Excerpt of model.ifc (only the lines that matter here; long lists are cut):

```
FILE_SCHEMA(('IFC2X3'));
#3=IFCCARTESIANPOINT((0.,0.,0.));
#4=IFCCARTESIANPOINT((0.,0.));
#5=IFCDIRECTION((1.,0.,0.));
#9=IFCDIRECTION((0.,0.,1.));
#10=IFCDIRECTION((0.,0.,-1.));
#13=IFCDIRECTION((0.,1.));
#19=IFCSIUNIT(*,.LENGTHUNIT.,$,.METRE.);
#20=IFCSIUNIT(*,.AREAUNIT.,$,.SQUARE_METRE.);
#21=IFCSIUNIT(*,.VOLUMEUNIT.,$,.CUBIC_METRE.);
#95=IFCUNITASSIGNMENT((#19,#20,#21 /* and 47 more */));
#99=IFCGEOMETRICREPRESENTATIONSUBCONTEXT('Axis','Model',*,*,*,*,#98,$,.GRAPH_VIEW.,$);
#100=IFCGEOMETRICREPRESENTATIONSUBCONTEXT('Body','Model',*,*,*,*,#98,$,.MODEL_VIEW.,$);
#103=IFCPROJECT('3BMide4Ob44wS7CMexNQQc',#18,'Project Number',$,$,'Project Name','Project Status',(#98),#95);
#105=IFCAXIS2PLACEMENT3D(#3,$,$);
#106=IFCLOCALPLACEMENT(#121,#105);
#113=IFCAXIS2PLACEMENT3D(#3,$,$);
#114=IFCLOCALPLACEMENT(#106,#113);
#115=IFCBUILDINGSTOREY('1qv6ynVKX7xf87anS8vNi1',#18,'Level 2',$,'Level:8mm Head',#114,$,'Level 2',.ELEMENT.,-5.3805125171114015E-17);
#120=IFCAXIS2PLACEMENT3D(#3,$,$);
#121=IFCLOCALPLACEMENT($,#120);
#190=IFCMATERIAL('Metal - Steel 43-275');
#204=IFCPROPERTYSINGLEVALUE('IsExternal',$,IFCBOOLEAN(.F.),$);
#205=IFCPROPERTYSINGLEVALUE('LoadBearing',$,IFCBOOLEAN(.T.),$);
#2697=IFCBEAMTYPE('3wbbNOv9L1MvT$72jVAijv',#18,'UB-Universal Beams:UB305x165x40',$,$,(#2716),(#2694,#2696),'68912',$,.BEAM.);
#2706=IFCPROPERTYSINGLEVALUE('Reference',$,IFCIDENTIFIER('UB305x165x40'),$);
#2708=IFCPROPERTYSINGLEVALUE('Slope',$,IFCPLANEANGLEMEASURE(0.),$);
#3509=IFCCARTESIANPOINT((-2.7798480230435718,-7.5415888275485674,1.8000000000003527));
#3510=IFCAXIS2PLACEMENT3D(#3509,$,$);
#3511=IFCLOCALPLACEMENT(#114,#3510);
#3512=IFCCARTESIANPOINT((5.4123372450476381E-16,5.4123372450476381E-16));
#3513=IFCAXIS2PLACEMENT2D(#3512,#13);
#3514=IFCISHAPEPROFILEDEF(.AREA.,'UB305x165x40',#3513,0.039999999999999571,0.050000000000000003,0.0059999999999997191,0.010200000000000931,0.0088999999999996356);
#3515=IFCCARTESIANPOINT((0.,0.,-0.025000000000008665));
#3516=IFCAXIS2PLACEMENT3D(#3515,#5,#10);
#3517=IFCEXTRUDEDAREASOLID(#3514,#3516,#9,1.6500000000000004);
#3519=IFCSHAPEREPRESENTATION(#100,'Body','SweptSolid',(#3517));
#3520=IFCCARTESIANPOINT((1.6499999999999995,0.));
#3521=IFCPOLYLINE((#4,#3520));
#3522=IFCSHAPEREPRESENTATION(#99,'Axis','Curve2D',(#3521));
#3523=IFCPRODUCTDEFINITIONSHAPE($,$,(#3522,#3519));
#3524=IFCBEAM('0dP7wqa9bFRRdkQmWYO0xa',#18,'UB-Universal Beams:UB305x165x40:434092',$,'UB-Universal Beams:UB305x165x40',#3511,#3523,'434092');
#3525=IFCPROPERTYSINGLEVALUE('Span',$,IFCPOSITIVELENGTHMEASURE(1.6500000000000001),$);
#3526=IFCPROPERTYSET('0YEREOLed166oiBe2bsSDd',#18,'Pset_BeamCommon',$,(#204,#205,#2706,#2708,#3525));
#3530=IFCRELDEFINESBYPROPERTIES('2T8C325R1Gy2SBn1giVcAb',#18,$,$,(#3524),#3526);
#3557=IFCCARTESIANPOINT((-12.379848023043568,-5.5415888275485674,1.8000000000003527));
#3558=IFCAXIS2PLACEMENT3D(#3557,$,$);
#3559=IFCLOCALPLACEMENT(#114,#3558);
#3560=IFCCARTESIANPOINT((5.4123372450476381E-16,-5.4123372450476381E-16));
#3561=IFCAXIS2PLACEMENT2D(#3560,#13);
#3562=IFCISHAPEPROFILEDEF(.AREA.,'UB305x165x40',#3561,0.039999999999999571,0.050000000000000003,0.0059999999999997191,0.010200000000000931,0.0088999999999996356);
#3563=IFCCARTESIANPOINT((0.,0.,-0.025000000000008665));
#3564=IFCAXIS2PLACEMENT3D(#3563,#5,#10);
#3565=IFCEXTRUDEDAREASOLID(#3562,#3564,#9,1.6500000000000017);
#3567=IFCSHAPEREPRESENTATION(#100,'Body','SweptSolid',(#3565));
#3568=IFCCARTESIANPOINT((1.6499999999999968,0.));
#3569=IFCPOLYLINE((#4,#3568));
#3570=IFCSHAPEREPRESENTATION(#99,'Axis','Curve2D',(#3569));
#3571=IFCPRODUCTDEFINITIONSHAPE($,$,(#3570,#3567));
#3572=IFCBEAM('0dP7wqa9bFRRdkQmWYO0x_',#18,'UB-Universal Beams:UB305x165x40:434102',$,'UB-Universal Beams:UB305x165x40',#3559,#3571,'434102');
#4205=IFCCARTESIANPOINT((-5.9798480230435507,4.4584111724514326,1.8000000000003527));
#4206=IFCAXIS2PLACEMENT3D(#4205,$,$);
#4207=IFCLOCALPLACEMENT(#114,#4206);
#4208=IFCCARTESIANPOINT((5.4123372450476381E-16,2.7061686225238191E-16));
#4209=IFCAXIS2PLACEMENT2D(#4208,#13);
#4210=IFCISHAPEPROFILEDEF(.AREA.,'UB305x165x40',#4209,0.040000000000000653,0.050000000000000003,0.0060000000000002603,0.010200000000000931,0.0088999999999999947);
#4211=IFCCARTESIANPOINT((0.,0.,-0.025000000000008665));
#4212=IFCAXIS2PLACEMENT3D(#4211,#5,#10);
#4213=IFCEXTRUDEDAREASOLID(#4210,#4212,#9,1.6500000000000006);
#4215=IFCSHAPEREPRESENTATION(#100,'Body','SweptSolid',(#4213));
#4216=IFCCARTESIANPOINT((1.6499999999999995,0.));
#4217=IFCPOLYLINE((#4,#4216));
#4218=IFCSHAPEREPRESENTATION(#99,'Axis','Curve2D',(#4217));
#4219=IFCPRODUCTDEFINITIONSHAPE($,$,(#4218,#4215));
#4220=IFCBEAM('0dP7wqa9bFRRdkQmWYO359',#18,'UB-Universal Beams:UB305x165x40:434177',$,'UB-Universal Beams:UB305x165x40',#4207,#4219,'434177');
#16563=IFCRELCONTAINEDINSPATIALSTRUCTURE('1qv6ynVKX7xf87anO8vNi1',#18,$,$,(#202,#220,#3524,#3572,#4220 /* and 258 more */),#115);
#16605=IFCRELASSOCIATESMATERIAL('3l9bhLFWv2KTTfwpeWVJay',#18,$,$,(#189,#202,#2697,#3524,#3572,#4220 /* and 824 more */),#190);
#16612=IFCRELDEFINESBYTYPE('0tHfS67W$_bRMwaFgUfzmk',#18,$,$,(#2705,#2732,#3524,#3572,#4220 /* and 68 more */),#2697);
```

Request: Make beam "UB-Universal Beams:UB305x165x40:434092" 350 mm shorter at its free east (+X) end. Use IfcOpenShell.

```python
import numpy as np
import ifcopenshell
import ifcopenshell.api.pset
import ifcopenshell.util.element
import ifcopenshell.util.representation

model = ifcopenshell.open("model.ifc")

member = model.by_guid("0dP7wqa9bFRRdkQmWYO0xa")
change = -0.35

# The extrusion runs towards the end named, so only its depth changes.
body = ifcopenshell.util.representation.get_representation(member, "Model", "Body")
solid = body.Items[0]
old_length = solid.Depth
solid.Depth += change

# Move the axis end point with it.
axis = next(r for r in member.Representation.Representations if r.RepresentationIdentifier == "Axis").Items[0]
start, end = (np.array(p.Coordinates) for p in axis.Points)
end = end + (end - start) / np.linalg.norm(end - start) * change
point = model.createIfcCartesianPoint(end.tolist())
axis.Points = [axis.Points[0], point]

# Update the stored length and volume.
pset = model.by_id(ifcopenshell.util.element.get_pset(member, "Pset_BeamCommon", should_inherit=False)["id"])
ifcopenshell.api.pset.edit_pset(model, pset=pset, properties={
    "Span": model.create_entity("IfcPositiveLengthMeasure", solid.Depth),
})

print(f"length {old_length:g} -> {solid.Depth:g}")

model.write("model_edited.ifc")
```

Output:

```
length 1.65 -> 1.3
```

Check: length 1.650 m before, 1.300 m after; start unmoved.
